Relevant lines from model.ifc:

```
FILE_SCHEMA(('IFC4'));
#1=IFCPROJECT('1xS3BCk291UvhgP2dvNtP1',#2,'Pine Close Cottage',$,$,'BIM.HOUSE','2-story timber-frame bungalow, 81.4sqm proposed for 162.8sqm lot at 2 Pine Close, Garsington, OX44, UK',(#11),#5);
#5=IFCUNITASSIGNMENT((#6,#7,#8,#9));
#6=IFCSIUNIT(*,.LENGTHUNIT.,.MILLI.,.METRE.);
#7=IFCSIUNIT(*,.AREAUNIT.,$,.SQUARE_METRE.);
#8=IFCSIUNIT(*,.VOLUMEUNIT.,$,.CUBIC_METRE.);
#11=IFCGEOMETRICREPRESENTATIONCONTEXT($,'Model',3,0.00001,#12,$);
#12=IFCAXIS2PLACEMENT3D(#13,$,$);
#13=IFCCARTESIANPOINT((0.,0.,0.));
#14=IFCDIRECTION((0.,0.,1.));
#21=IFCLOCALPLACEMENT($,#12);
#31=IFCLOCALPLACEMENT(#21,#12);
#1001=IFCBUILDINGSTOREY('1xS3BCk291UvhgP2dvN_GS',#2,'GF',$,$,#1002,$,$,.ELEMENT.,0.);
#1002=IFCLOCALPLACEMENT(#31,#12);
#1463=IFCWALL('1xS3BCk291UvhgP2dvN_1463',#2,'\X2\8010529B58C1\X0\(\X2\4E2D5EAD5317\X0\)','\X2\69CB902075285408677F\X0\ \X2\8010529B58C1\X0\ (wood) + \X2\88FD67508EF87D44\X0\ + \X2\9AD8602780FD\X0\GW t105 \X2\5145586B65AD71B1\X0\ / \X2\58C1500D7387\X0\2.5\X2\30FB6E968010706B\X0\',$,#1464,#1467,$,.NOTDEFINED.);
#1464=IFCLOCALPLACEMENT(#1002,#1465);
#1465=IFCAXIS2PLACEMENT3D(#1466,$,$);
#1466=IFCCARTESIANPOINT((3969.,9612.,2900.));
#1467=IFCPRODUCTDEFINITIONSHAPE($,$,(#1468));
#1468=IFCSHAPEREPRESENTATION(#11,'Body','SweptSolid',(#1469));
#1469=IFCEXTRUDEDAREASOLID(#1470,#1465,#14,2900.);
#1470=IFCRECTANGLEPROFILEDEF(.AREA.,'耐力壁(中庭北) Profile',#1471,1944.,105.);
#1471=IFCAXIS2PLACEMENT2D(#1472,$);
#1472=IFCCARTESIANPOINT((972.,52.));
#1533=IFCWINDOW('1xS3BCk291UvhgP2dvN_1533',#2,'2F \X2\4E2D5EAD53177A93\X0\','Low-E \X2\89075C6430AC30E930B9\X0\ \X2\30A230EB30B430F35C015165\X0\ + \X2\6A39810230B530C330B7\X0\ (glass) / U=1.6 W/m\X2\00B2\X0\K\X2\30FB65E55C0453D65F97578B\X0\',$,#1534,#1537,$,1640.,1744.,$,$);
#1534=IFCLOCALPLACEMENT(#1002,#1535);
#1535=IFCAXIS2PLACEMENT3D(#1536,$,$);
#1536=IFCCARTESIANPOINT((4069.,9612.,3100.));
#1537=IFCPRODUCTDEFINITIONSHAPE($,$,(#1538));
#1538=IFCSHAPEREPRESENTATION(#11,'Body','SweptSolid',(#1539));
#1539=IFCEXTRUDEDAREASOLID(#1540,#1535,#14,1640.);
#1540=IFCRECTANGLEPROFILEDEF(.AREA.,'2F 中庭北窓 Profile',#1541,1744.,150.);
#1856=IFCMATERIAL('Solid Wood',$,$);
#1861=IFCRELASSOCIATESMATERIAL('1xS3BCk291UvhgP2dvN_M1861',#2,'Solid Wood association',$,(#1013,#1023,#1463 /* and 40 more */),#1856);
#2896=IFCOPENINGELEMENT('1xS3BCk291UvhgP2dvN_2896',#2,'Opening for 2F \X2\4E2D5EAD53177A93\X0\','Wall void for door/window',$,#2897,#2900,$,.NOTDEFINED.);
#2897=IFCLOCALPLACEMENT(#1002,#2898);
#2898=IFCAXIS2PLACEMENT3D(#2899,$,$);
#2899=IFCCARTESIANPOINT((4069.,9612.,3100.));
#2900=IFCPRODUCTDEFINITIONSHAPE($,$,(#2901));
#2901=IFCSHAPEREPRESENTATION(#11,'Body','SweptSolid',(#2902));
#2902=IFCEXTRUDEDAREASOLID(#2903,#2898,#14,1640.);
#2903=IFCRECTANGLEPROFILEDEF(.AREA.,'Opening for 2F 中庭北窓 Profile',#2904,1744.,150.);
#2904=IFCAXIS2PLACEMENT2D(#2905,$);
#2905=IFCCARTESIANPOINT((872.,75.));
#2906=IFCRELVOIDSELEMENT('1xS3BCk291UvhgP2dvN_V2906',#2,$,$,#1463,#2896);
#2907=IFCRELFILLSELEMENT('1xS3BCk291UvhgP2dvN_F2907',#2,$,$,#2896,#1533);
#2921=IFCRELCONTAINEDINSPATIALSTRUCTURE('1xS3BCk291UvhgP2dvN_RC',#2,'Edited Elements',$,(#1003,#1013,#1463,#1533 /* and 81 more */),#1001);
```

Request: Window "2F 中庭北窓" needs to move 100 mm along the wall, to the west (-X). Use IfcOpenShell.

```python
import ifcopenshell
import ifcopenshell.api.geometry
import ifcopenshell.util.placement

model = ifcopenshell.open("model.ifc")

window = model.by_guid("1xS3BCk291UvhgP2dvN_1533")
opening = window.FillsVoids[0].RelatingOpeningElement
wall = opening.VoidsElements[0].RelatingBuildingElement

wall_matrix = ifcopenshell.util.placement.get_local_placement(wall.ObjectPlacement)
shift = wall_matrix[:3, 0] * -100.0
before = ifcopenshell.util.placement.get_local_placement(window.ObjectPlacement)[:3, 3].copy()

# The window is not placed relative to its opening, so move both.
for product in (opening, window):
    matrix = ifcopenshell.util.placement.get_local_placement(product.ObjectPlacement)
    matrix[:3, 3] += shift
    ifcopenshell.api.geometry.edit_object_placement(model, product=product, matrix=matrix, is_si=False)

after = ifcopenshell.util.placement.get_local_placement(window.ObjectPlacement)[:3, 3]
print("window moved by", (after - before).round(3) + 0.0)

model.write("model-out.ifc")
```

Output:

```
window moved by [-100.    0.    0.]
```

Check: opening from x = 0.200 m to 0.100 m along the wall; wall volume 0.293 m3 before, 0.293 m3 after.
